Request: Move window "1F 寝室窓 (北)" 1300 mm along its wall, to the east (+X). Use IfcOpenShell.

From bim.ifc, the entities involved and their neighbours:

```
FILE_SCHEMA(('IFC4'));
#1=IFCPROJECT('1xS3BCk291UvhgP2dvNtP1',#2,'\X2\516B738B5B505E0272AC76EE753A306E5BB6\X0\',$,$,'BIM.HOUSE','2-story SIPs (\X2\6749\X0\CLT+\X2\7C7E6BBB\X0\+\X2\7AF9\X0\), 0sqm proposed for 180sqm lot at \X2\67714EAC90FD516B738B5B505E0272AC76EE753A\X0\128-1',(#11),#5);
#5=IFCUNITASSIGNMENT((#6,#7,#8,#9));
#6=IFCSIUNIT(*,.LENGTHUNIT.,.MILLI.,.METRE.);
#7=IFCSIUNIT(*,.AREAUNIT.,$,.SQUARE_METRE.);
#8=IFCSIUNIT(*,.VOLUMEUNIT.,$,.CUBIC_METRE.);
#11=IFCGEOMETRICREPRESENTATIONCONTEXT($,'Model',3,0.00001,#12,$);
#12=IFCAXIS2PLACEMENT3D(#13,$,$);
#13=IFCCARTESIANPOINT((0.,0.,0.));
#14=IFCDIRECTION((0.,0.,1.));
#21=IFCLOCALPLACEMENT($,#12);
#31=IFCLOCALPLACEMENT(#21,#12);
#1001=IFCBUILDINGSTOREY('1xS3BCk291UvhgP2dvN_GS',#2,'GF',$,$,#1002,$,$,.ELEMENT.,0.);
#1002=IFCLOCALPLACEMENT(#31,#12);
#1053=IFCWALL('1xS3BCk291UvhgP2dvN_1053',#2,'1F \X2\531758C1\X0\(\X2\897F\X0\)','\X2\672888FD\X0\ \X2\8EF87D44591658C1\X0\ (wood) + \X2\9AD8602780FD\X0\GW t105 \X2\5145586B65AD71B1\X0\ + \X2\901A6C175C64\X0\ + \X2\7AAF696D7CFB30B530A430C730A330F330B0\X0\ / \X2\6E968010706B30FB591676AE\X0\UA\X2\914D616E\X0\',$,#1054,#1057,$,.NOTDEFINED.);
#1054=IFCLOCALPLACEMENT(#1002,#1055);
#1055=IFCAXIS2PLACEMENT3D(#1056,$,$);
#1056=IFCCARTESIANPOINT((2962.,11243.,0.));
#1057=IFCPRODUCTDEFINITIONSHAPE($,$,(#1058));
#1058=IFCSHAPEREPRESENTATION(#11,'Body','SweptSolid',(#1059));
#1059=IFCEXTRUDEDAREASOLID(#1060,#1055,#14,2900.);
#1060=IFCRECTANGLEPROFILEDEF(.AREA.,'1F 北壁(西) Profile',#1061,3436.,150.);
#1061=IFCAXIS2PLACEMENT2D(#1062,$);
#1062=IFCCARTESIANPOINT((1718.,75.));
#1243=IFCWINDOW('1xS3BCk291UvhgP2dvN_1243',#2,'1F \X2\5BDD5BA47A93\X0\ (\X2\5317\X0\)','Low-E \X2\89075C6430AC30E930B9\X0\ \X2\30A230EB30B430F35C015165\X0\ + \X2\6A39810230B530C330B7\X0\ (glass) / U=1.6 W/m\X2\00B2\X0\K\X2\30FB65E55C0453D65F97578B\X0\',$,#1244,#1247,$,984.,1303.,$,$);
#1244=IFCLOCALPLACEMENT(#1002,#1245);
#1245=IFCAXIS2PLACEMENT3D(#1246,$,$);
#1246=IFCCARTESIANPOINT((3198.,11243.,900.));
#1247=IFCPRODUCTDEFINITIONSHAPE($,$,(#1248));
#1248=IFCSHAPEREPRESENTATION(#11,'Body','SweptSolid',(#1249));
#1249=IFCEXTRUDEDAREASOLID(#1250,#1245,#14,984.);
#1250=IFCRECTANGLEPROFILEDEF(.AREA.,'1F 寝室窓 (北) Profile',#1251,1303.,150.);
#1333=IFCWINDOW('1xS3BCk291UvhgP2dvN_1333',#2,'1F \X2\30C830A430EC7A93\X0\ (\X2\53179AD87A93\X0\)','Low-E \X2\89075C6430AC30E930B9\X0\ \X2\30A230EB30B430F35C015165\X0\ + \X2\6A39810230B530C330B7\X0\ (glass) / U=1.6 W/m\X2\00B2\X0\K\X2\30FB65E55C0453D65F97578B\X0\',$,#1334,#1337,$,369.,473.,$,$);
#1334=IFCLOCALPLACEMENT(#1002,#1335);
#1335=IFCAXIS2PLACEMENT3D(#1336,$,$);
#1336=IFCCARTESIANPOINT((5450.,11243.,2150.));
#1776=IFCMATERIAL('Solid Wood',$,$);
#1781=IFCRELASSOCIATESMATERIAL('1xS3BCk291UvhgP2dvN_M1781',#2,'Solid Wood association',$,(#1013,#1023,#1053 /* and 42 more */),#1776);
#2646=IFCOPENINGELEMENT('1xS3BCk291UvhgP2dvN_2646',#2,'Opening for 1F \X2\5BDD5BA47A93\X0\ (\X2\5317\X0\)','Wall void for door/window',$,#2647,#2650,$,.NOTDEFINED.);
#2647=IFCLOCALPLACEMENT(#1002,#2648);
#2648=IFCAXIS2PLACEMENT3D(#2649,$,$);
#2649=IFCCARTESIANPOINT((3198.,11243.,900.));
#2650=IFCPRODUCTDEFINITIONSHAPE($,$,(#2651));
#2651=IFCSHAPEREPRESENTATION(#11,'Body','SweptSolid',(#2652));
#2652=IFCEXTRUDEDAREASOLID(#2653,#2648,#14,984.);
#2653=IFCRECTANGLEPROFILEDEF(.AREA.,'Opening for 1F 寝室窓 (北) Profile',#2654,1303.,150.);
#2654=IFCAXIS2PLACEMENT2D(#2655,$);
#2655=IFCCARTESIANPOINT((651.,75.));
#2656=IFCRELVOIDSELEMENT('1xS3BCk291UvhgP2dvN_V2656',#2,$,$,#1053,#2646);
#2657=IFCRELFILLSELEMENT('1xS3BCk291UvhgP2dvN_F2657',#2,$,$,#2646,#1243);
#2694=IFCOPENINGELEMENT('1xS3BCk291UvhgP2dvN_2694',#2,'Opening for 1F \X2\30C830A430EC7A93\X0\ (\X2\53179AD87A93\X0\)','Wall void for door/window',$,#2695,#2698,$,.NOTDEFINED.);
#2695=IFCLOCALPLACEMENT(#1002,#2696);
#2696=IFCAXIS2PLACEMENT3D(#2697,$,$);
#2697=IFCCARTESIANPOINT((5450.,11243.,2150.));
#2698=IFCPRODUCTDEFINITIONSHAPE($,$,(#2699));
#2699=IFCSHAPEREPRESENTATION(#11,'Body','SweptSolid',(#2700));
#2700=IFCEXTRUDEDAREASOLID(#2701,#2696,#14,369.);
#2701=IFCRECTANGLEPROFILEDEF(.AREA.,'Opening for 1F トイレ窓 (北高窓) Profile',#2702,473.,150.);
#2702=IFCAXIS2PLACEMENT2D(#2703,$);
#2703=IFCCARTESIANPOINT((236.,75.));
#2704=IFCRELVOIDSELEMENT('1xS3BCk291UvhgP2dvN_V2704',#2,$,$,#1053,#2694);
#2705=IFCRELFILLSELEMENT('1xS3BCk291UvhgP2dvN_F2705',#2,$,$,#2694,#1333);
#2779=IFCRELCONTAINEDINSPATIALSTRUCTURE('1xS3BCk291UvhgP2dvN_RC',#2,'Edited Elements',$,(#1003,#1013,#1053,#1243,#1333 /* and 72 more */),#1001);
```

```python
import ifcopenshell
import ifcopenshell.api.geometry
import ifcopenshell.util.placement

model = ifcopenshell.open("bim.ifc")

window = model.by_guid("1xS3BCk291UvhgP2dvN_1243")
opening = window.FillsVoids[0].RelatingOpeningElement
wall = opening.VoidsElements[0].RelatingBuildingElement

wall_matrix = ifcopenshell.util.placement.get_local_placement(wall.ObjectPlacement)
shift = wall_matrix[:3, 0] * 1300.0
before = ifcopenshell.util.placement.get_local_placement(window.ObjectPlacement)[:3, 3].copy()

# The window is not placed relative to its opening, so move both.
for product in (opening, window):
    matrix = ifcopenshell.util.placement.get_local_placement(product.ObjectPlacement)
    matrix[:3, 3] += shift
    ifcopenshell.api.geometry.edit_object_placement(model, product=product, matrix=matrix, is_si=False)

after = ifcopenshell.util.placement.get_local_placement(window.ObjectPlacement)[:3, 3]
print("window moved by", (after - before).round(3) + 0.0)

model.write("bim-out.ifc")
```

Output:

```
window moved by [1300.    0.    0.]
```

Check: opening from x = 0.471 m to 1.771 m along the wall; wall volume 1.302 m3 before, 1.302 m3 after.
